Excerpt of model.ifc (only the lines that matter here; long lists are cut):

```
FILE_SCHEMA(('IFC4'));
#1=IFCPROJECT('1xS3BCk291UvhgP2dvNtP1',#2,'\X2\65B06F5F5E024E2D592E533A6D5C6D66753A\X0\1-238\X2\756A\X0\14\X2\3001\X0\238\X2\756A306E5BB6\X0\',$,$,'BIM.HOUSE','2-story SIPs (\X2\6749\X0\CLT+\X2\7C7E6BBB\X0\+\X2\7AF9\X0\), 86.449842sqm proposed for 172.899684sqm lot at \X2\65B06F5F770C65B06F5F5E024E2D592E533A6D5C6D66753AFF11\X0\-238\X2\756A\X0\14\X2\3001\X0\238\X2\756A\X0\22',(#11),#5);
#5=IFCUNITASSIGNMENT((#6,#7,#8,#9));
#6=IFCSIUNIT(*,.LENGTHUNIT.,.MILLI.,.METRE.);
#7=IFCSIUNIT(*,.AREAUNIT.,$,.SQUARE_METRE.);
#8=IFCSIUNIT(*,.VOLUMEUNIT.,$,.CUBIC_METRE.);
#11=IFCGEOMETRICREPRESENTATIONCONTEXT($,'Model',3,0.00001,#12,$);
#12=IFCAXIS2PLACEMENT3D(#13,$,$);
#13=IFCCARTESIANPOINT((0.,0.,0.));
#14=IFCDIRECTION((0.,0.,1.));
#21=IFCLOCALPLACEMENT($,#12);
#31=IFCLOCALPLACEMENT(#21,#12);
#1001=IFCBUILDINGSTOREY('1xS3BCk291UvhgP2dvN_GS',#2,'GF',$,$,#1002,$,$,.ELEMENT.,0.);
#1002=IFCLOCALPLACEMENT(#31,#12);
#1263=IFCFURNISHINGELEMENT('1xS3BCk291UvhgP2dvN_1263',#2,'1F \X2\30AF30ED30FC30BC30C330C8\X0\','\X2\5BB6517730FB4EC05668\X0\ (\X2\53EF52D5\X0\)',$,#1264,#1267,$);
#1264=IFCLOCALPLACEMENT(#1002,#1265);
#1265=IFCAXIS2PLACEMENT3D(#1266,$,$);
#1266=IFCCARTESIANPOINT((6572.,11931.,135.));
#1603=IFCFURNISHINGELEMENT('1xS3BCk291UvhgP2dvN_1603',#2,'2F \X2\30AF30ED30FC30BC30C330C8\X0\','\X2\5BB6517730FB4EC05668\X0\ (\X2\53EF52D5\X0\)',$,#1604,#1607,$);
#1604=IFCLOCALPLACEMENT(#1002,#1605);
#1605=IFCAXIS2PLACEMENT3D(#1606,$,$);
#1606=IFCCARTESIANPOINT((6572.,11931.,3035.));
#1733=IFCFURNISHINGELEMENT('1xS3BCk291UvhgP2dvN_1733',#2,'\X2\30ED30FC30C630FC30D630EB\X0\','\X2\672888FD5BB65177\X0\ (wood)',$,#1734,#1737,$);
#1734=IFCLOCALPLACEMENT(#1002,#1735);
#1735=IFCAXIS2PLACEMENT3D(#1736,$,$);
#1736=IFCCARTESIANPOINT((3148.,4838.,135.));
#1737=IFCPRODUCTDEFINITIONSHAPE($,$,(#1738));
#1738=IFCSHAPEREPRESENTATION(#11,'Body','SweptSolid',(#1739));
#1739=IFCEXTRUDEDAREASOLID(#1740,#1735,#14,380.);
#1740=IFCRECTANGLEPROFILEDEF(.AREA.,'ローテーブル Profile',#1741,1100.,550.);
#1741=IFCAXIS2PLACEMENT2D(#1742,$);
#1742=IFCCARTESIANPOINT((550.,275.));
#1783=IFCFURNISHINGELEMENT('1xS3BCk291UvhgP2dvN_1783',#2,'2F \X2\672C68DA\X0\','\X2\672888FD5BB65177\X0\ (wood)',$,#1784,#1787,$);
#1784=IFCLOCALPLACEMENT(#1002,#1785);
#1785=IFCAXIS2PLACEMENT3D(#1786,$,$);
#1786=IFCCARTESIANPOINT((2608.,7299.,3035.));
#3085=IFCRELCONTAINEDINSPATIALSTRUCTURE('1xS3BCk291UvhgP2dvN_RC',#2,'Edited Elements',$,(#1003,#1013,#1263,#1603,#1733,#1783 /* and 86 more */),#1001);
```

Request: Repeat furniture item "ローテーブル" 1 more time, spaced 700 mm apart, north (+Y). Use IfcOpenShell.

```python
import numpy as np
import ifcopenshell
import ifcopenshell.api.geometry
import ifcopenshell.api.root
import ifcopenshell.util.element
import ifcopenshell.util.placement
import ifcopenshell.util.unit

model = ifcopenshell.open("model.ifc")
unit_scale = ifcopenshell.util.unit.calculate_unit_scale(model)


def reuse_history(source, copy):
    """copy_class also copies each property set's owner history, people and application; keep the originals."""
    for rel in copy.IsDefinedBy:
        if rel.is_a("IfcRelDefinesByProperties") and (history := rel.RelatingPropertyDefinition.OwnerHistory):
            rel.RelatingPropertyDefinition.OwnerHistory = source.OwnerHistory
            ifcopenshell.util.element.remove_deep2(model, history)


source = model.by_guid("1xS3BCk291UvhgP2dvN_1733")
base = ifcopenshell.util.placement.get_local_placement(source.ObjectPlacement)
step = np.array([0.0, 1.0, 0.0]) * 0.7 / unit_scale

for i in range(1, 2):
    copy = ifcopenshell.api.root.copy_class(model, product=source)
    copy.Representation = ifcopenshell.util.element.copy_deep(
        model, source.Representation, exclude=["IfcGeometricRepresentationContext", "IfcRepresentationMap"]
    )
    reuse_history(source, copy)
    matrix = base.copy()
    matrix[:3, 3] += i * step
    print("added at", matrix[:3, 3].round(3) + 0.0)
    ifcopenshell.api.geometry.edit_object_placement(model, product=copy, matrix=matrix, is_si=False)

model.write("model_edited.ifc")
```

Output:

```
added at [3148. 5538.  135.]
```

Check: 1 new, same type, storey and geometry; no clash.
